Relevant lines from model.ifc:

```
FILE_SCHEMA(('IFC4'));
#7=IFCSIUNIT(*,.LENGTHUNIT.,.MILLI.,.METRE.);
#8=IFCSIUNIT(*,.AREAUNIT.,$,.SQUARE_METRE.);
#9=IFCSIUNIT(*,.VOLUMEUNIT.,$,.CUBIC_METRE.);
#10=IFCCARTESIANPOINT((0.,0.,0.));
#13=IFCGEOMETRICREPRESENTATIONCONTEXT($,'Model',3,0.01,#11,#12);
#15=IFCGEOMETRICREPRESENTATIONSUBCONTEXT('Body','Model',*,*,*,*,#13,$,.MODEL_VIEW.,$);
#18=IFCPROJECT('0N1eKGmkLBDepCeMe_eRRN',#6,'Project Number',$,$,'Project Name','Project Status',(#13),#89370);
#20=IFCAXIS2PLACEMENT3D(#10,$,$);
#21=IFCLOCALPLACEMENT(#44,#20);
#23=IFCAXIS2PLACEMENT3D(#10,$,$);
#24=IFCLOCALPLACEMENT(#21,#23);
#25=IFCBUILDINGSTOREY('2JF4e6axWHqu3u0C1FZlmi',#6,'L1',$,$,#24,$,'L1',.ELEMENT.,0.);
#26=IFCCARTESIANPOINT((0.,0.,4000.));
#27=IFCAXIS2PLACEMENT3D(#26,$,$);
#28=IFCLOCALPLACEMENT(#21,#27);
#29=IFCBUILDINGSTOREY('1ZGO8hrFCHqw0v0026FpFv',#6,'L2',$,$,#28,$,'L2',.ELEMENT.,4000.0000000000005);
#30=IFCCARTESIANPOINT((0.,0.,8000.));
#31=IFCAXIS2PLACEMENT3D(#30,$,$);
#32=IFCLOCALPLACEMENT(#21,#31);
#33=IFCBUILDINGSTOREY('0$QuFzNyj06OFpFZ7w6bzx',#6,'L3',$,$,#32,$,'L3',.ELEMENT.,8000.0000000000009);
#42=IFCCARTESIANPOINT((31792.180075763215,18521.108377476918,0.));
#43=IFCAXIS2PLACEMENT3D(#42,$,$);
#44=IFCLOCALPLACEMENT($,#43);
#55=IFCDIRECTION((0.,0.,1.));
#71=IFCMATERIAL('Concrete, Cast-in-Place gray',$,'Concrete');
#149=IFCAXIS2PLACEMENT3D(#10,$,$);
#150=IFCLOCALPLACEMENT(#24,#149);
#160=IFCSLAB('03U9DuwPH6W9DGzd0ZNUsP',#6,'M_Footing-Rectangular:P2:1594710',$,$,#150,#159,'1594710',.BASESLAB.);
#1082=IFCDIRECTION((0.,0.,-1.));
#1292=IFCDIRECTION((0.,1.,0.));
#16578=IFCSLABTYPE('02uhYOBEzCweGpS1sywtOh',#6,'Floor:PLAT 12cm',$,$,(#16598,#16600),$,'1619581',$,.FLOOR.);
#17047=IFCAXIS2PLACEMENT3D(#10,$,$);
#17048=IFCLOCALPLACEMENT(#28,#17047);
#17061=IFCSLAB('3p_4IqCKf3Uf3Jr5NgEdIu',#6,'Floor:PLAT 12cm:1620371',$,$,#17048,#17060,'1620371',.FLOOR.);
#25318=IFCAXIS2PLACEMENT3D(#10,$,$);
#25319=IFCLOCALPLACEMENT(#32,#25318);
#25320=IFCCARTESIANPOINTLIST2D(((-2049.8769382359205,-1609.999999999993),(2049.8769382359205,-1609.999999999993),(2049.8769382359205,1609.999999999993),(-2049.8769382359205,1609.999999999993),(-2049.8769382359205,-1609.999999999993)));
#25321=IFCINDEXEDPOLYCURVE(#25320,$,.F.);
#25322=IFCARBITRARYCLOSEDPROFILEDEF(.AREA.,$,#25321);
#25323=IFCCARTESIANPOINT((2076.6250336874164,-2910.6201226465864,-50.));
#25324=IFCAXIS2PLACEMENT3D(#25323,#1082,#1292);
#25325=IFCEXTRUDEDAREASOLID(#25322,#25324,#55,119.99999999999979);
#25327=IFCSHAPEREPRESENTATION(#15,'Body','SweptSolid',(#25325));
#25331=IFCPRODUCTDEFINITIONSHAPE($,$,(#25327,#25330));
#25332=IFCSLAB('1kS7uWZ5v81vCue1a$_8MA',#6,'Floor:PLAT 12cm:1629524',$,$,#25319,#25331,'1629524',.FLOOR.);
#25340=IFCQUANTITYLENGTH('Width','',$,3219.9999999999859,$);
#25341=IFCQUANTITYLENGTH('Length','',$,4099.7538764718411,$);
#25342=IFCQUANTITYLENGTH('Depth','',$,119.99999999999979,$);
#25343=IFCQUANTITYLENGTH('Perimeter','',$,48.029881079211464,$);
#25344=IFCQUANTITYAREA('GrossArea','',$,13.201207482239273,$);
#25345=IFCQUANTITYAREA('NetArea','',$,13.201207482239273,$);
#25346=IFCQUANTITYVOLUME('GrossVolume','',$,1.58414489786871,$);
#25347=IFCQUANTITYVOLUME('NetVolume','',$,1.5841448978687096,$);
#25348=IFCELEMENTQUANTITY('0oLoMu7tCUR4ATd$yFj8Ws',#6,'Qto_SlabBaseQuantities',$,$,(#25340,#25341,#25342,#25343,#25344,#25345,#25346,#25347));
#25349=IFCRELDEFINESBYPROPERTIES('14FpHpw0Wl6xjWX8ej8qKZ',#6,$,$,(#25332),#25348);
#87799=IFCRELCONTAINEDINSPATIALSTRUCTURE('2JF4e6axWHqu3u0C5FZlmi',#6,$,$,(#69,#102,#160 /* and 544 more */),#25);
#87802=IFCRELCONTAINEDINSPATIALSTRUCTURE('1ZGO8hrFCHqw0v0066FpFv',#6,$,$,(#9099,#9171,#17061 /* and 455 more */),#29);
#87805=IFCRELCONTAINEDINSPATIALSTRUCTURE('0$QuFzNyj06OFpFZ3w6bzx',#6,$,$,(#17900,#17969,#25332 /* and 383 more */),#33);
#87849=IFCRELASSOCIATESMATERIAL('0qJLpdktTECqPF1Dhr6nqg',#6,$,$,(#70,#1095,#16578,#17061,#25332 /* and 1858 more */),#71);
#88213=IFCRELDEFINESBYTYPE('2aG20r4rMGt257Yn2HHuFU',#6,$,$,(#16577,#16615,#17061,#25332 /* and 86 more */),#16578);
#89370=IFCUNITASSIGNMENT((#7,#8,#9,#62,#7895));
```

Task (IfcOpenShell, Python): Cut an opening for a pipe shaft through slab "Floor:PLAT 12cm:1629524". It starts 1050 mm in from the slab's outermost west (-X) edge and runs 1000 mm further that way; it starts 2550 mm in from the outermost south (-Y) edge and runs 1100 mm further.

```python
import numpy as np
import ifcopenshell
import ifcopenshell.api.feature
import ifcopenshell.api.geometry
import ifcopenshell.api.pset
import ifcopenshell.api.root
import ifcopenshell.geom
import ifcopenshell.util.element
import ifcopenshell.util.placement
import ifcopenshell.util.representation
import ifcopenshell.util.shape
import ifcopenshell.util.unit

model = ifcopenshell.open("model.ifc")
unit_scale = ifcopenshell.util.unit.calculate_unit_scale(model)
area_scale = ifcopenshell.util.unit.calculate_unit_scale(model, "AREAUNIT")
volume_scale = ifcopenshell.util.unit.calculate_unit_scale(model, "VOLUMEUNIT")
settings = ifcopenshell.geom.settings()


def volume(element):
    """Net volume in cubic metres, openings subtracted."""
    shape = ifcopenshell.geom.create_shape(settings, element)
    return ifcopenshell.util.shape.get_volume(shape.geometry)


slab = model.by_guid("1kS7uWZ5v81vCue1a$_8MA")
before = volume(slab)

# Extent in the slab's own axes, in metres. The edges named are its -X and -Y sides.
slab_shape = ifcopenshell.geom.create_shape(settings, slab)
vertices = ifcopenshell.util.shape.get_vertices(slab_shape.geometry)
x_min, y_min, bottom = vertices.min(axis=0)
top = vertices[:, 2].max()

opening = ifcopenshell.api.root.create_entity(model, ifc_class="IfcOpeningElement", name="Pipe shaft opening", predefined_type="OPENING")
context = ifcopenshell.util.representation.get_context(model, "Model", "Body", "MODEL_VIEW")
width, depth = 1, 1.1
outline = [(0.0, 0.0), (width, 0.0), (width, depth), (0.0, depth), (0.0, 0.0)]
# Overshoot both faces by 50 mm so the cut is clean.
shape = ifcopenshell.api.geometry.add_slab_representation(
    model, context=context, depth=top - bottom + 0.1, polyline=outline
)
ifcopenshell.api.geometry.assign_representation(model, product=opening, representation=shape)

matrix = ifcopenshell.util.placement.get_local_placement(slab.ObjectPlacement)
matrix[:, 3] = matrix @ np.append(np.array([x_min + 1.05, y_min + 2.55, bottom - 0.05]) / unit_scale, 1.0)
ifcopenshell.api.geometry.edit_object_placement(model, product=opening, matrix=matrix, is_si=False)
ifcopenshell.api.feature.add_feature(model, feature=opening, element=slab)

after = volume(slab)

# Update the slab's stored quantities.
qto = model.by_id(ifcopenshell.util.element.get_pset(slab, "Qto_SlabBaseQuantities", should_inherit=False)["id"])
ifcopenshell.api.pset.edit_qto(model, qto=qto, properties={
    "NetArea": after / (top - bottom) / area_scale,
    "NetVolume": after / volume_scale,
})

print(f"slab volume {before:.3f} -> {after:.3f} m3")

model.write("model_rev.ifc")
```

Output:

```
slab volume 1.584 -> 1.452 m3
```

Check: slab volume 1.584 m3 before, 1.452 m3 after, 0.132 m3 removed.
